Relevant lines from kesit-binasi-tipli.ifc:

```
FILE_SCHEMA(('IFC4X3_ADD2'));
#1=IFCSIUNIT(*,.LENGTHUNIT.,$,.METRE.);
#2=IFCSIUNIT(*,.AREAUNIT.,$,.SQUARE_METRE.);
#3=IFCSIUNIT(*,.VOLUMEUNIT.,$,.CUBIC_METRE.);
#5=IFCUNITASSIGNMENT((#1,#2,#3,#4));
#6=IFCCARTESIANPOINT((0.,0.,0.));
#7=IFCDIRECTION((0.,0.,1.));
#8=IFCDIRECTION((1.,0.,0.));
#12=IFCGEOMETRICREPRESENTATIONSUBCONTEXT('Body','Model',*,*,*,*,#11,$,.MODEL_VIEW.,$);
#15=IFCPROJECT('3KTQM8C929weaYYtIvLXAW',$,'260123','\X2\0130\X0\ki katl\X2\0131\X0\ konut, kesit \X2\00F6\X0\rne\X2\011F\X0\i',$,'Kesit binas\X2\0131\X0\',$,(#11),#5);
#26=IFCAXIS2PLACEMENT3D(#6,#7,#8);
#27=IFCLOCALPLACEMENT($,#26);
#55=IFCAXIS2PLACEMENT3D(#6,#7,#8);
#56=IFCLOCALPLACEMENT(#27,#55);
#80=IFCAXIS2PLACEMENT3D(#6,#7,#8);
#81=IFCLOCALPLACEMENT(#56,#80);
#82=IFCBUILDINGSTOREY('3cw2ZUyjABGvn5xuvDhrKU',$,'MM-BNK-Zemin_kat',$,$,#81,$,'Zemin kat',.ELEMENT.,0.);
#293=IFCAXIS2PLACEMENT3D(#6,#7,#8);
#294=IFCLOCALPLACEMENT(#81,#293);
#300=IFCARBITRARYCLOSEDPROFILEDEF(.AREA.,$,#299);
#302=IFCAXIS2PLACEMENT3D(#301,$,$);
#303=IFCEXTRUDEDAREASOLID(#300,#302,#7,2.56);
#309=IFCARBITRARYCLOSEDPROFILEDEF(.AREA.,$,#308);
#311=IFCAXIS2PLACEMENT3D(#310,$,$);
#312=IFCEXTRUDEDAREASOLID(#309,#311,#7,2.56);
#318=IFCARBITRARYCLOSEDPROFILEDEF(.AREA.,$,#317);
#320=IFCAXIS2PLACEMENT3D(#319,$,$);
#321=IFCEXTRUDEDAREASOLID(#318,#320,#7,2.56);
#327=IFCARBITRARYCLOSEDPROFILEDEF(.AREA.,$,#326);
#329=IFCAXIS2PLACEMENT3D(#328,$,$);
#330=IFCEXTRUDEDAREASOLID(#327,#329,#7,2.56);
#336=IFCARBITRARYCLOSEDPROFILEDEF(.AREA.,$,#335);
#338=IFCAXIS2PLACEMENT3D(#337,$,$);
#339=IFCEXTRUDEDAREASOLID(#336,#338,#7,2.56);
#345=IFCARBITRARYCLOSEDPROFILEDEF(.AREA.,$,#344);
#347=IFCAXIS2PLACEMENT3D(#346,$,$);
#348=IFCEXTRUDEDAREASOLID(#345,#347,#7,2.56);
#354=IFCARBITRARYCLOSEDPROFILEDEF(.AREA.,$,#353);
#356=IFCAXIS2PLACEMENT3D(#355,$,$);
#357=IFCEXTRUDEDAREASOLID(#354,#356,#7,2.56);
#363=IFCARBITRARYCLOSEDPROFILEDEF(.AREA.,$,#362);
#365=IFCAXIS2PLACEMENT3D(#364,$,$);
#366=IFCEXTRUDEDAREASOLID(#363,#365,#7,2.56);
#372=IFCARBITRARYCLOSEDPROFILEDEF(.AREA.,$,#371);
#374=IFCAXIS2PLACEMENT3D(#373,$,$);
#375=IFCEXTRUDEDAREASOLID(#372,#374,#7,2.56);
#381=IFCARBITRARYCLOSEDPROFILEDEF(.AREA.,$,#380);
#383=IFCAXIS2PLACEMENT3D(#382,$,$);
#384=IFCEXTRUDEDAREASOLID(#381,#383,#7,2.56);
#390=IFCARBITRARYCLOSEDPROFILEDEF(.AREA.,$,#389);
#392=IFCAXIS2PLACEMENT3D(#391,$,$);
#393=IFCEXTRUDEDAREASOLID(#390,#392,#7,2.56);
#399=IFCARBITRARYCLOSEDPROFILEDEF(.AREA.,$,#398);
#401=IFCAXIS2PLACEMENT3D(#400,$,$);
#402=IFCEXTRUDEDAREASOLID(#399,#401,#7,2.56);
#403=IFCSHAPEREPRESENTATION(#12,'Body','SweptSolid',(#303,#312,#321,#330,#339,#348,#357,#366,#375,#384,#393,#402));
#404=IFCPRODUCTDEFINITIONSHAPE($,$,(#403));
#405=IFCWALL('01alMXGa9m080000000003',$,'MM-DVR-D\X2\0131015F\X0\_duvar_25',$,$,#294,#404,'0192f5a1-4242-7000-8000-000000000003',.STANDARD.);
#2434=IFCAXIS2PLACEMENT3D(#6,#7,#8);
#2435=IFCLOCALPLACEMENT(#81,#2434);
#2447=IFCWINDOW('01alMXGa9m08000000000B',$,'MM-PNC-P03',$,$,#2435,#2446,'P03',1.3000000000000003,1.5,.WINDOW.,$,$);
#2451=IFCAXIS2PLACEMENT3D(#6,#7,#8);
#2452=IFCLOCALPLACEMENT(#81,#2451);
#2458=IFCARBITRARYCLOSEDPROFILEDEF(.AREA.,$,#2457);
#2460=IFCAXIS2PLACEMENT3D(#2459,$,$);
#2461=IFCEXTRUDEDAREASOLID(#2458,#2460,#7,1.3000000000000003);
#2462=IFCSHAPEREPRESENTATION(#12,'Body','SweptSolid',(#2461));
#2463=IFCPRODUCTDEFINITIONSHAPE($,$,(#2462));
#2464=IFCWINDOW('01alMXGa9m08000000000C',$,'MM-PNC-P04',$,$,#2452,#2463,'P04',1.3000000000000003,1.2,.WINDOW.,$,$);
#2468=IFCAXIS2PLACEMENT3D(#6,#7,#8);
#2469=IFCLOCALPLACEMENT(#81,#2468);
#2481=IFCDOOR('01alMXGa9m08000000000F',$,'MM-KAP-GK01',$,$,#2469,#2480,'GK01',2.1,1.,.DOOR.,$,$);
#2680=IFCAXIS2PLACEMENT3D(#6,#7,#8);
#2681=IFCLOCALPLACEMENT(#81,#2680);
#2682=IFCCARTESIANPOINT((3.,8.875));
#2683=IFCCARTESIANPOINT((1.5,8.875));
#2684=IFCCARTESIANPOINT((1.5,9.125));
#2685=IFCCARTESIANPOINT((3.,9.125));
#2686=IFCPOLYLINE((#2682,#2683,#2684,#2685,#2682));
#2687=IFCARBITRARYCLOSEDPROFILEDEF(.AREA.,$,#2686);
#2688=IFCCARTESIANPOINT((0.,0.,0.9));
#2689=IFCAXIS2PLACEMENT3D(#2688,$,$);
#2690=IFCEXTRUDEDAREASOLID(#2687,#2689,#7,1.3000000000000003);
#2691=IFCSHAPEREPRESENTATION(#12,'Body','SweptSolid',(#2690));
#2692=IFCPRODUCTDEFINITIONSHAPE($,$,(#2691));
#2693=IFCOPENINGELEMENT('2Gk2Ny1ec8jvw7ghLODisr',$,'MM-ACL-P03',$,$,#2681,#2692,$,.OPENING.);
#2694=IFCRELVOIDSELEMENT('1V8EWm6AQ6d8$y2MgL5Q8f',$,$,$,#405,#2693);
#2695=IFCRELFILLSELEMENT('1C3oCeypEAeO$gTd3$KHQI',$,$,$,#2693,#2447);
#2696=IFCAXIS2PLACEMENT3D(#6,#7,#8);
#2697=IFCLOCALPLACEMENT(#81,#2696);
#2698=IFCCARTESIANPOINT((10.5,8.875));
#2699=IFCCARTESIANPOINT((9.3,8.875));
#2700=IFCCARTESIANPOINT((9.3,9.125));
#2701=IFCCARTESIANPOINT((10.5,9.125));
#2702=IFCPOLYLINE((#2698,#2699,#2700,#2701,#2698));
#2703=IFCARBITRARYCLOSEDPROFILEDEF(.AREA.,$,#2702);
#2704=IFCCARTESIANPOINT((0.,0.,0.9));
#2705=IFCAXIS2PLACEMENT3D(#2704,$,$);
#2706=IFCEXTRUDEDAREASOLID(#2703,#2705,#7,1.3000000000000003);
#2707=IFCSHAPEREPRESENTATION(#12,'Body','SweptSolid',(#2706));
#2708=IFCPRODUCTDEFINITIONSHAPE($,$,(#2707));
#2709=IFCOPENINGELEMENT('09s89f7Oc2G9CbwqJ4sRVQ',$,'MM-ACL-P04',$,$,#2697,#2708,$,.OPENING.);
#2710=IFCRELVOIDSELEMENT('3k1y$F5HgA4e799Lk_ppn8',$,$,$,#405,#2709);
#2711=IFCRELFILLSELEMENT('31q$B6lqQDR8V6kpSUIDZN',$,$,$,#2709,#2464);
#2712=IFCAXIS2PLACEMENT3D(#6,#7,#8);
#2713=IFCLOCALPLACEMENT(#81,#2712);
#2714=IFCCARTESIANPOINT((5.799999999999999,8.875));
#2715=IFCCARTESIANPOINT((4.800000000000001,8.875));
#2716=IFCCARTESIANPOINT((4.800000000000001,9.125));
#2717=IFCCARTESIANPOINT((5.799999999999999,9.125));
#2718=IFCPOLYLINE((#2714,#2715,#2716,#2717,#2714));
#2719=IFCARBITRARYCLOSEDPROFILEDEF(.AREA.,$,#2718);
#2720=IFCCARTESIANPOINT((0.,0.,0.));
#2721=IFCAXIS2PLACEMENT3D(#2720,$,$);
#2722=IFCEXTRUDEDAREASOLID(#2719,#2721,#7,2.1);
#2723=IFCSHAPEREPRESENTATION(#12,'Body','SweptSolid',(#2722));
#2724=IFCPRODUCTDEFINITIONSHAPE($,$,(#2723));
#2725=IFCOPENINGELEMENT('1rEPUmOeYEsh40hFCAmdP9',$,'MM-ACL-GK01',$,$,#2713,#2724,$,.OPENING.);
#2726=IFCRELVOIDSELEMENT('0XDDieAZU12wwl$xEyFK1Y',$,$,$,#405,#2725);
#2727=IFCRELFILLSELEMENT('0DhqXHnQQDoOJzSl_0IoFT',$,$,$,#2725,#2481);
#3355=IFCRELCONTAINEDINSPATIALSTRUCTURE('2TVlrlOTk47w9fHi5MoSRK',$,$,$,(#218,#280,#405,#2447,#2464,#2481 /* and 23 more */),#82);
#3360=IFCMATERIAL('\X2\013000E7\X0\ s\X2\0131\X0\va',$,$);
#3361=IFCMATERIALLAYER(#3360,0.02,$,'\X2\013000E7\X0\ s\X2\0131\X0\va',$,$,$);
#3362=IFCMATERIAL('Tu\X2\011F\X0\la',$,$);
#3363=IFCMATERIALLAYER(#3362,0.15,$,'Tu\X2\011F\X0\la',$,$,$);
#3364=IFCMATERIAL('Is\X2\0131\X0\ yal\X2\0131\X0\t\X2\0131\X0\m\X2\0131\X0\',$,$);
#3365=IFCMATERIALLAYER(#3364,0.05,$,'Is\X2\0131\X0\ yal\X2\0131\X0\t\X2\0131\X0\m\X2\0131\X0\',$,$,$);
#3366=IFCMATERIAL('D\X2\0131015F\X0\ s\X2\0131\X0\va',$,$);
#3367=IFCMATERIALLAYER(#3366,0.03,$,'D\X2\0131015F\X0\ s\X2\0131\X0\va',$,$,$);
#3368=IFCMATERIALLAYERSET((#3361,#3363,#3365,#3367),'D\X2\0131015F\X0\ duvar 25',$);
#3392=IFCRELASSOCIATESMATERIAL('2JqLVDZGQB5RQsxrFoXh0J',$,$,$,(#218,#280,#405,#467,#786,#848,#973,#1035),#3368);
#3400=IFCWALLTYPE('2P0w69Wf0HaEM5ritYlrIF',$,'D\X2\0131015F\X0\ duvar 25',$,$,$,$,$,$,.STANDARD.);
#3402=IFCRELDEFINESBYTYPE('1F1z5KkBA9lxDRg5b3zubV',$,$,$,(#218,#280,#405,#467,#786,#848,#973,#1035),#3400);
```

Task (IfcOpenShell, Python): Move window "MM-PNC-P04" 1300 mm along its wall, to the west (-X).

```python
import ifcopenshell
import ifcopenshell.api.geometry
import ifcopenshell.util.placement

model = ifcopenshell.open("kesit-binasi-tipli.ifc")

window = model.by_id(2464)
opening = window.FillsVoids[0].RelatingOpeningElement
wall = opening.VoidsElements[0].RelatingBuildingElement

wall_matrix = ifcopenshell.util.placement.get_local_placement(wall.ObjectPlacement)
shift = wall_matrix[:3, 0] * -1.3
before = ifcopenshell.util.placement.get_local_placement(window.ObjectPlacement)[:3, 3].copy()

# The window is not placed relative to its opening, so move both.
for product in (opening, window):
    matrix = ifcopenshell.util.placement.get_local_placement(product.ObjectPlacement)
    matrix[:3, 3] += shift
    ifcopenshell.api.geometry.edit_object_placement(model, product=product, matrix=matrix, is_si=False)

after = ifcopenshell.util.placement.get_local_placement(window.ObjectPlacement)[:3, 3]
print("window moved by", (after - before).round(3) + 0.0)

model.write("kesit-binasi-tipli_edited.ifc")
```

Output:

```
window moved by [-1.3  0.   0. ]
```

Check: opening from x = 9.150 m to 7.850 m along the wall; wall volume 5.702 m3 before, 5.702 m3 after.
